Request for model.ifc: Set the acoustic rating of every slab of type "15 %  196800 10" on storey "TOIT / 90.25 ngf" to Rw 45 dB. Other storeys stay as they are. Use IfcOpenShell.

First a look at what the model holds.

```python
import ifcopenshell
import ifcopenshell.util.element

model = ifcopenshell.open("model.ifc")
print(model.schema)
storey = next(s for s in model.by_type("IfcBuildingStorey") if s.Name == "TOIT / 90.25 ngf")
slabs = [e for e in ifcopenshell.util.element.get_decomposition(storey) if e.is_a("IfcSlab")]
seen = {}
for e in slabs:
    element_type = ifcopenshell.util.element.get_type(e)
    key = (element_type.Name if element_type != e and element_type else None, ifcopenshell.util.element.get_pset(e, "Pset_SlabCommon", "AcousticRating"))
    seen[key] = seen.get(key, 0) + 1
for (name, value), count in sorted(seen.items(), key=str):
    print(count, "x", name, "|", value)
```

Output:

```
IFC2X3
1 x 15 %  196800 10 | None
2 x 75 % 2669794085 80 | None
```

```python
import ifcopenshell
import ifcopenshell.api.pset
import ifcopenshell.util.element

model = ifcopenshell.open("model.ifc")

storey = next(s for s in model.by_type("IfcBuildingStorey") if s.Name == "TOIT / 90.25 ngf")
slabs = [e for e in ifcopenshell.util.element.get_decomposition(storey) if e.is_a("IfcSlab")]

count = 0
for e in slabs:
    element_type = ifcopenshell.util.element.get_type(e)
    if element_type in (None, e) or element_type.Name != "15 %  196800 10":
        continue
    # add_pset returns the element's existing set when there is one.
    pset = ifcopenshell.api.pset.add_pset(model, product=e, name="Pset_SlabCommon")
    ifcopenshell.api.pset.edit_pset(model, pset=pset, properties={"AcousticRating": "Rw 45 dB"})
    count += 1

print(count, "slabs updated")

model.write("model-out.ifc")
```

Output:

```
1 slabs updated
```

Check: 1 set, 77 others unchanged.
